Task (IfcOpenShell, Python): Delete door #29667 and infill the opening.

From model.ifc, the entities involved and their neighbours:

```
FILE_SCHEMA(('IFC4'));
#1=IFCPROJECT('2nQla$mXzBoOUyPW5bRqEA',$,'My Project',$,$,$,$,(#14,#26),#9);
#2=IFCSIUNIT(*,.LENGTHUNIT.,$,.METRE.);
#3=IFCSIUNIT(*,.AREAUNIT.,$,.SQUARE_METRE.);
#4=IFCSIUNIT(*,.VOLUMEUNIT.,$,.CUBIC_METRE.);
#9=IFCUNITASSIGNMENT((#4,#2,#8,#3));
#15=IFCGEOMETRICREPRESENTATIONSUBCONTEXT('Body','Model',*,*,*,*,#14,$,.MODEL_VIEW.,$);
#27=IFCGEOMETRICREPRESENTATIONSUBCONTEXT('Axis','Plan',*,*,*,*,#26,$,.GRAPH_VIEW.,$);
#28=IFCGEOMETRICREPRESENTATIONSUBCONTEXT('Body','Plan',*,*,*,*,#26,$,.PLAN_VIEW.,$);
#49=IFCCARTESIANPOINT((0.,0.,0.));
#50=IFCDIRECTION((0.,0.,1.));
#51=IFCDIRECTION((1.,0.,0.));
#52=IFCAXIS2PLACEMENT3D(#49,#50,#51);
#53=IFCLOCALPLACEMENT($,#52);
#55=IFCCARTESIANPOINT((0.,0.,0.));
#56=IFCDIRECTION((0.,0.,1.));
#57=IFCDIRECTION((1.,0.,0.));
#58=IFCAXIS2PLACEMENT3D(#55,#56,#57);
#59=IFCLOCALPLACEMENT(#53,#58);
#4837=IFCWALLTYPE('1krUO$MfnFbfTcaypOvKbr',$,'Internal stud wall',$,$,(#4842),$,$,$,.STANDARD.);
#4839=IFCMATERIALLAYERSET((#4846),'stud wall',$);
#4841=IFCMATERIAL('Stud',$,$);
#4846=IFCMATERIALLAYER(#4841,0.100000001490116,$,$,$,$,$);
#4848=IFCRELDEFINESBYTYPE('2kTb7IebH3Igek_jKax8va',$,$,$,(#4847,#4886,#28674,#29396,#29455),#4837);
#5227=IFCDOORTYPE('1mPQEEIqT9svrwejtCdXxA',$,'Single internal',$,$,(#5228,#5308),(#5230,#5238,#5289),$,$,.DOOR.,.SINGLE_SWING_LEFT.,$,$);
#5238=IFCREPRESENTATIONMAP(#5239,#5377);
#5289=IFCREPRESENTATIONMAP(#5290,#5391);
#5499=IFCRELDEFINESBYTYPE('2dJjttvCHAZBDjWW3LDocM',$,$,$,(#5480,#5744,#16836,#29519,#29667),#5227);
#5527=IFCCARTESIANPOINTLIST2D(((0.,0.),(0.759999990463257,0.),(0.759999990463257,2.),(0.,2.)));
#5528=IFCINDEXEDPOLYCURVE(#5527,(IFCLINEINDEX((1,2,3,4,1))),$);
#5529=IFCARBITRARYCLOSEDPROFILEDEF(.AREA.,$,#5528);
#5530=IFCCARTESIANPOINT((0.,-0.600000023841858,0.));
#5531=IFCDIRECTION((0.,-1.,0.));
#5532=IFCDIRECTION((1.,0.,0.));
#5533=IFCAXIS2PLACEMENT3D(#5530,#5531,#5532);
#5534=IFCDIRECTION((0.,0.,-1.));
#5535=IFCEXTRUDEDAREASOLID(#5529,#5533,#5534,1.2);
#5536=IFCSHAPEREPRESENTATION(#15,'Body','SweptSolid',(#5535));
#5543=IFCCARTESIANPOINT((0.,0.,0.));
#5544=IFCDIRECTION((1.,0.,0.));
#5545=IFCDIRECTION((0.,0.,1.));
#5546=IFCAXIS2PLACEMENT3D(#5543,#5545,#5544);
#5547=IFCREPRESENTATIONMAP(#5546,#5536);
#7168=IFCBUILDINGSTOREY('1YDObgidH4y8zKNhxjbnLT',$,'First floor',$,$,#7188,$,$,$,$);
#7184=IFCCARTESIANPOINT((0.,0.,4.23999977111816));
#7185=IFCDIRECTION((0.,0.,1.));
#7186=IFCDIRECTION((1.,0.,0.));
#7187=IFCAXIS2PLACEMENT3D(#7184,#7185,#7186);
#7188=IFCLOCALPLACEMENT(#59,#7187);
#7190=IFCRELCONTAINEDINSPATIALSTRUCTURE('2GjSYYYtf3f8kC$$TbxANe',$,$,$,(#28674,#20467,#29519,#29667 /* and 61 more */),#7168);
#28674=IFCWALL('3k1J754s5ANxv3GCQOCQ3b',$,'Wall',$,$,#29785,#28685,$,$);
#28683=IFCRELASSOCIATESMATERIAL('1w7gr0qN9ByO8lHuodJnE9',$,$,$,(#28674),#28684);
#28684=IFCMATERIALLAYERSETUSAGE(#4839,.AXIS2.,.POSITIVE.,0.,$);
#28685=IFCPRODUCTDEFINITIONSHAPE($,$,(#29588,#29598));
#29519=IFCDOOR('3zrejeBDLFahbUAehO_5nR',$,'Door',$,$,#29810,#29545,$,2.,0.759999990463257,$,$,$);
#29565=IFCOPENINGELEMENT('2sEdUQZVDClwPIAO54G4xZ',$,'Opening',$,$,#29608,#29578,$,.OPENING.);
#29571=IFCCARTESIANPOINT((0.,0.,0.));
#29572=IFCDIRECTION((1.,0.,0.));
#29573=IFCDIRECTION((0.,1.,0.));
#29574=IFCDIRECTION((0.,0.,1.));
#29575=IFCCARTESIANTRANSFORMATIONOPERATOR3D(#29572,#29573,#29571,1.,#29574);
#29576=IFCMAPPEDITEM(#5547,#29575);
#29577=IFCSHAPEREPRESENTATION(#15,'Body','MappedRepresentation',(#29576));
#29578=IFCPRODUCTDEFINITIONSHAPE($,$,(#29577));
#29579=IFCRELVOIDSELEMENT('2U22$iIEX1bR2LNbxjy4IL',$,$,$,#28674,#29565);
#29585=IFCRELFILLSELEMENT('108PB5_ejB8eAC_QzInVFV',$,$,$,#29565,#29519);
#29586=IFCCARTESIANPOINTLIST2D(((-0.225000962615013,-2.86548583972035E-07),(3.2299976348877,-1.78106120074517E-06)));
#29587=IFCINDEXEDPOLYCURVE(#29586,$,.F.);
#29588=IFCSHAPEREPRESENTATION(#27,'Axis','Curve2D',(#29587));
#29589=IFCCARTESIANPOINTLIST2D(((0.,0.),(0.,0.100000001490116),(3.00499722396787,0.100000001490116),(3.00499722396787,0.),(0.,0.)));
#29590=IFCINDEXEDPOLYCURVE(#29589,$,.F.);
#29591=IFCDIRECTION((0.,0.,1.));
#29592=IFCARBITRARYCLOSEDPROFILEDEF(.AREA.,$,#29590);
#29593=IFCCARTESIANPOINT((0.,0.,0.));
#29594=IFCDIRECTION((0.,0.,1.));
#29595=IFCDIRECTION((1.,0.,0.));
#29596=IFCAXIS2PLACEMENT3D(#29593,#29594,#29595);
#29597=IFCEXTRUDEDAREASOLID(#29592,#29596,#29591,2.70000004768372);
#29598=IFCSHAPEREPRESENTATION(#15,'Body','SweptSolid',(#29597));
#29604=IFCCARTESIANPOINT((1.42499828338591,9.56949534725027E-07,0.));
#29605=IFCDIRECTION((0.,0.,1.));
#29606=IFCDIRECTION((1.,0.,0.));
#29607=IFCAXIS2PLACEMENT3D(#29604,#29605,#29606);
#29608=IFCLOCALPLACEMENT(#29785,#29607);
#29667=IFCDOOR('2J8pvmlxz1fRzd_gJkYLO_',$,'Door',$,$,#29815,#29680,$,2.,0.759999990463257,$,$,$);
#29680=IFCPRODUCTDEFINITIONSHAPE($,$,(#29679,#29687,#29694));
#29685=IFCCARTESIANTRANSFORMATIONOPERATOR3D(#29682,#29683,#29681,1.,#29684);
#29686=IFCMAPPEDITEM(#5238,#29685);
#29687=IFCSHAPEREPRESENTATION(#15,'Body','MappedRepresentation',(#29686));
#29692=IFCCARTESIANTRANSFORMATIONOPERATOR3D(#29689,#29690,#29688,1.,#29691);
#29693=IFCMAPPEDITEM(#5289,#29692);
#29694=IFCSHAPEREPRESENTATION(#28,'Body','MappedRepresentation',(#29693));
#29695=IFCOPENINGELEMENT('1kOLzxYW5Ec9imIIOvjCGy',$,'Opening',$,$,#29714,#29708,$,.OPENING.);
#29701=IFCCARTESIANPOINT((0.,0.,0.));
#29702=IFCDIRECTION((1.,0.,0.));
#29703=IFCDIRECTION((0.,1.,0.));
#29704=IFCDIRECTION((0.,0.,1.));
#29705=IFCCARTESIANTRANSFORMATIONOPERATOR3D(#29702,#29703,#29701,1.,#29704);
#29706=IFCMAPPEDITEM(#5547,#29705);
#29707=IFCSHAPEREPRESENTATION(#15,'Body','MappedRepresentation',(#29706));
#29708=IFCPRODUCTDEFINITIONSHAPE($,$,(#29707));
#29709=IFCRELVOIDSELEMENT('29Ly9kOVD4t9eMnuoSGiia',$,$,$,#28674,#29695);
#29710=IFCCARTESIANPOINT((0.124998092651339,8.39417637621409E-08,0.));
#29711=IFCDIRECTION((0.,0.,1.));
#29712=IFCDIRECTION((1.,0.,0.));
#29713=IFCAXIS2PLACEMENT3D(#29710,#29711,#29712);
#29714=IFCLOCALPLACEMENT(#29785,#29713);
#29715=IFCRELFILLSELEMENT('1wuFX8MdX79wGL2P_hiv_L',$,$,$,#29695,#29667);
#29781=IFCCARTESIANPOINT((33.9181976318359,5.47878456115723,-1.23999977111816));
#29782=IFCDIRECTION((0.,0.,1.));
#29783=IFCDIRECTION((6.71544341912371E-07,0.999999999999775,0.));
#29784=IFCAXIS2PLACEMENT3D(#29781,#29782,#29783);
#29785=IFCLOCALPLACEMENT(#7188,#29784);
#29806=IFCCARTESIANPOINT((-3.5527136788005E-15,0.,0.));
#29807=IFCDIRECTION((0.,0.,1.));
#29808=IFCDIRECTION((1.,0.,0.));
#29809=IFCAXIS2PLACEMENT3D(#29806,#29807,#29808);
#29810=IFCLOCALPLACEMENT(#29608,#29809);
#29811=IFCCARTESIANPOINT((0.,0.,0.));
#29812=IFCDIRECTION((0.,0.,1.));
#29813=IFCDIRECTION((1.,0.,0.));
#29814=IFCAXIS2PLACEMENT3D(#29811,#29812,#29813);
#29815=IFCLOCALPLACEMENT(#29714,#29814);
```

```python
import ifcopenshell
import ifcopenshell.api.feature
import ifcopenshell.api.root
import ifcopenshell.geom
import ifcopenshell.util.shape

model = ifcopenshell.open("model.ifc")
settings = ifcopenshell.geom.settings()


def volume(element):
    """Net volume in cubic metres, openings subtracted."""
    shape = ifcopenshell.geom.create_shape(settings, element)
    return ifcopenshell.util.shape.get_volume(shape.geometry)


door = model.by_guid("2J8pvmlxz1fRzd_gJkYLO_")
opening = door.FillsVoids[0].RelatingOpeningElement
wall = opening.VoidsElements[0].RelatingBuildingElement
before = volume(wall)

ifcopenshell.api.root.remove_product(model, product=door)
ifcopenshell.api.feature.remove_feature(model, feature=opening)

after = volume(wall)

print(f"wall volume {before:.3f} -> {after:.3f} m3")

model.write("model_updated.ifc")
```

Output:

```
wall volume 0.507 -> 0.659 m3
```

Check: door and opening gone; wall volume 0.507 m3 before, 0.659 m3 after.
